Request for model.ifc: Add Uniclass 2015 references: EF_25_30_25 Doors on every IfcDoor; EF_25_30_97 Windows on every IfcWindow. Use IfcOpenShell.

First a look at what the model holds.

```python
import ifcopenshell

model = ifcopenshell.open("model.ifc")
print(model.schema)
print("classifications:", [c.Name for c in model.by_type("IfcClassification")])
for ifc_class in ("IfcDoor", "IfcRoof", "IfcStair", "IfcWall", "IfcWindow"):
    print(ifc_class, len(model.by_type(ifc_class)))
```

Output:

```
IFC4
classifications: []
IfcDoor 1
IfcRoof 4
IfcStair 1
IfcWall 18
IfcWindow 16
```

```python
import ifcopenshell
import ifcopenshell.api.classification

model = ifcopenshell.open("model.ifc")

system = ifcopenshell.api.classification.add_classification(model, classification="Uniclass 2015")

codes = {
    "IfcDoor": ("EF_25_30_25", "Doors"),
    "IfcWindow": ("EF_25_30_97", "Windows"),
}
for ifc_class, (code, name) in codes.items():
    products = model.by_type(ifc_class)
    ifcopenshell.api.classification.add_reference(
        model, products=products, classification=system, identification=code, name=name
    )
    print(code, len(products))

model.write("model_rev.ifc")
```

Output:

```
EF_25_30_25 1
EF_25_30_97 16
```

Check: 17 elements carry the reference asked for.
